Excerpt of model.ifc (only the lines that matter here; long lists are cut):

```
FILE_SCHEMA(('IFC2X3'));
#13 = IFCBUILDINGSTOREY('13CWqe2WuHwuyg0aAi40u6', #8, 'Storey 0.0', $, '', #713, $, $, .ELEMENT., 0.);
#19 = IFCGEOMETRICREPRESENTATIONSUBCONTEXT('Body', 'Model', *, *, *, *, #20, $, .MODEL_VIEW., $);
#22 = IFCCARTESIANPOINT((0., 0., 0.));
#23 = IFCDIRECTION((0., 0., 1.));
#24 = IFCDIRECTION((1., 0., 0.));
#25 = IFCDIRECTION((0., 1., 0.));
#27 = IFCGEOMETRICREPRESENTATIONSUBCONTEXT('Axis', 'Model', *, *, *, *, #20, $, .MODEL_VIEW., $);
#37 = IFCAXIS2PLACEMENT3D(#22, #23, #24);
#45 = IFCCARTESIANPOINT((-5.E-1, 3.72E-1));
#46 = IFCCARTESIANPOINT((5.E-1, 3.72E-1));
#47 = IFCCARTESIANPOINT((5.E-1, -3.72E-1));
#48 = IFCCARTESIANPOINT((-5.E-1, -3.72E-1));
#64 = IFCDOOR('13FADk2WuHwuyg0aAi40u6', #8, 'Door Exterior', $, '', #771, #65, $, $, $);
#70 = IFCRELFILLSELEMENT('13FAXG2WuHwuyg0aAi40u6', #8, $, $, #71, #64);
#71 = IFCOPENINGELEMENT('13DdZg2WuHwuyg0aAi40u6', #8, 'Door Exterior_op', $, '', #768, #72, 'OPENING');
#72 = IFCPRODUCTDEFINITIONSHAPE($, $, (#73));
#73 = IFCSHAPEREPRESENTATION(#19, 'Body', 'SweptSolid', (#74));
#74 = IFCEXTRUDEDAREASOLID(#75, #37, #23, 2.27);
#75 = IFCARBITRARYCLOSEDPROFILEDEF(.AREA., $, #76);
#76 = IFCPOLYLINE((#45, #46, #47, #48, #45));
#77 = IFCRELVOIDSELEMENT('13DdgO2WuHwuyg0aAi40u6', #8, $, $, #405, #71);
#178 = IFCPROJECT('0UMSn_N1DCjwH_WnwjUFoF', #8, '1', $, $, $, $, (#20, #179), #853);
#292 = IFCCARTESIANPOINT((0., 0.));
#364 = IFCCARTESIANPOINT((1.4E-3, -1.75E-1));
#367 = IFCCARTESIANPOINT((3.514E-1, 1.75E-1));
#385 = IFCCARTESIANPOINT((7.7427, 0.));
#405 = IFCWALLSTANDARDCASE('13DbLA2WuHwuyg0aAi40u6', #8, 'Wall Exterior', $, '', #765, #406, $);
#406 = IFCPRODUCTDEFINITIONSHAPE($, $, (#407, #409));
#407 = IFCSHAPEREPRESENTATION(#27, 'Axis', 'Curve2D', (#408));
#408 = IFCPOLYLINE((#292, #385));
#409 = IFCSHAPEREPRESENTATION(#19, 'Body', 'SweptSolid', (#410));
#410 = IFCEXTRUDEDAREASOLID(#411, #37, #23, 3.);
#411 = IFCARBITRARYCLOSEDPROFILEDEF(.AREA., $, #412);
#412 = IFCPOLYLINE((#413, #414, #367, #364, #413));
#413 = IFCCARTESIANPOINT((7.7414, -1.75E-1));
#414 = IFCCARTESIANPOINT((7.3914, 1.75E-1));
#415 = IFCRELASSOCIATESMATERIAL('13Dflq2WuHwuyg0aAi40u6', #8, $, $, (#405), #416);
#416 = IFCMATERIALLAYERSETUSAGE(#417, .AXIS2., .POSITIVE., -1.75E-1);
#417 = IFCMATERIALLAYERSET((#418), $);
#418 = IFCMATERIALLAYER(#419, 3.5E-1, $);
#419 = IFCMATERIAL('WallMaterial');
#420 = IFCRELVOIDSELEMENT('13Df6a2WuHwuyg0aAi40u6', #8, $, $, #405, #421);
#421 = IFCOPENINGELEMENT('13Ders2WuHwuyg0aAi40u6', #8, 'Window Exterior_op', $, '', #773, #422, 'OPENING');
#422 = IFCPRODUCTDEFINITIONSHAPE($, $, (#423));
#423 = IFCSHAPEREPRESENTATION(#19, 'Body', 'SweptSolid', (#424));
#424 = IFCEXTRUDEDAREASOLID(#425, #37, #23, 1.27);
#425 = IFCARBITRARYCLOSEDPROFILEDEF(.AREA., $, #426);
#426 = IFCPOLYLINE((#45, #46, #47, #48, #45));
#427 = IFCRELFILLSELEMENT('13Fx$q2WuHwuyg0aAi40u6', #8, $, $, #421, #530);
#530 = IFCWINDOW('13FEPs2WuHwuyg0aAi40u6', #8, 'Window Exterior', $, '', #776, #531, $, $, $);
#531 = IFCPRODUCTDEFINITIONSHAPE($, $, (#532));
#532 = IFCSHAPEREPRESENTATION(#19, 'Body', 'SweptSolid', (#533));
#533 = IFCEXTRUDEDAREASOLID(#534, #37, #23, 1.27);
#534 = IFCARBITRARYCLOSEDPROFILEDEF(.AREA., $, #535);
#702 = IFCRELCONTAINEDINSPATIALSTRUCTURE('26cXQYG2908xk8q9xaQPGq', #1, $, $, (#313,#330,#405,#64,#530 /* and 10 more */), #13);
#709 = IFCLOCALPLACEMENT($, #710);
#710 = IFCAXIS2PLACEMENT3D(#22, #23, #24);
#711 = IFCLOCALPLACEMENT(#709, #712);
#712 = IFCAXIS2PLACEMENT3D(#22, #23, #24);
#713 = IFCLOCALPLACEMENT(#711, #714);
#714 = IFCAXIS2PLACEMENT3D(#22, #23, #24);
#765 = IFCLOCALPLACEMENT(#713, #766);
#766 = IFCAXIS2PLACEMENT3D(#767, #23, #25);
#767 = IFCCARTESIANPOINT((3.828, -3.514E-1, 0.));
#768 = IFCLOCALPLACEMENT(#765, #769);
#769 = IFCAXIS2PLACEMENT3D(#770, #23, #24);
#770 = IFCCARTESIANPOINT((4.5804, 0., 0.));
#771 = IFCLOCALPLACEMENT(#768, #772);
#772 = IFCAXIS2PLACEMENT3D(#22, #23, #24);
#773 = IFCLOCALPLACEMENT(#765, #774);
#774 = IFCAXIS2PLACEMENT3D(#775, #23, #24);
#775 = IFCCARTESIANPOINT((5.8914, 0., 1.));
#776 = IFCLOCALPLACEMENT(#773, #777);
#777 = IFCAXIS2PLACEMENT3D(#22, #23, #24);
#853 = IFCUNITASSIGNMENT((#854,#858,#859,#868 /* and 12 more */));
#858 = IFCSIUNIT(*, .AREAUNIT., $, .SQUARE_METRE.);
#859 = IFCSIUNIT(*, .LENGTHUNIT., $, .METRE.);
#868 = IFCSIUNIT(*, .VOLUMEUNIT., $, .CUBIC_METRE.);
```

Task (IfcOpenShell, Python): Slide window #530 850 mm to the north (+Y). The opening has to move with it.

```python
import ifcopenshell
import ifcopenshell.api.geometry
import ifcopenshell.util.placement
import ifcopenshell.util.unit

model = ifcopenshell.open("model.ifc")
unit_scale = ifcopenshell.util.unit.calculate_unit_scale(model)

window = model.by_guid("13FEPs2WuHwuyg0aAi40u6")
opening = window.FillsVoids[0].RelatingOpeningElement
wall = opening.VoidsElements[0].RelatingBuildingElement

wall_matrix = ifcopenshell.util.placement.get_local_placement(wall.ObjectPlacement)
shift = wall_matrix[:3, 0] * 0.85 / unit_scale
before = ifcopenshell.util.placement.get_local_placement(window.ObjectPlacement)[:3, 3].copy()

# The window is placed relative to its opening, so it follows when the opening moves.
matrix = ifcopenshell.util.placement.get_local_placement(opening.ObjectPlacement)
matrix[:3, 3] += shift
ifcopenshell.api.geometry.edit_object_placement(
    model, product=opening, matrix=matrix, is_si=False, should_transform_children=True
)

after = ifcopenshell.util.placement.get_local_placement(window.ObjectPlacement)[:3, 3]
print("window moved by", (after - before).round(3) + 0.0)

model.write("model_edited.ifc")
```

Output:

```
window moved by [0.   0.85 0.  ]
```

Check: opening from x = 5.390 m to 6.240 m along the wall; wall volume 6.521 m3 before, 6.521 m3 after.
